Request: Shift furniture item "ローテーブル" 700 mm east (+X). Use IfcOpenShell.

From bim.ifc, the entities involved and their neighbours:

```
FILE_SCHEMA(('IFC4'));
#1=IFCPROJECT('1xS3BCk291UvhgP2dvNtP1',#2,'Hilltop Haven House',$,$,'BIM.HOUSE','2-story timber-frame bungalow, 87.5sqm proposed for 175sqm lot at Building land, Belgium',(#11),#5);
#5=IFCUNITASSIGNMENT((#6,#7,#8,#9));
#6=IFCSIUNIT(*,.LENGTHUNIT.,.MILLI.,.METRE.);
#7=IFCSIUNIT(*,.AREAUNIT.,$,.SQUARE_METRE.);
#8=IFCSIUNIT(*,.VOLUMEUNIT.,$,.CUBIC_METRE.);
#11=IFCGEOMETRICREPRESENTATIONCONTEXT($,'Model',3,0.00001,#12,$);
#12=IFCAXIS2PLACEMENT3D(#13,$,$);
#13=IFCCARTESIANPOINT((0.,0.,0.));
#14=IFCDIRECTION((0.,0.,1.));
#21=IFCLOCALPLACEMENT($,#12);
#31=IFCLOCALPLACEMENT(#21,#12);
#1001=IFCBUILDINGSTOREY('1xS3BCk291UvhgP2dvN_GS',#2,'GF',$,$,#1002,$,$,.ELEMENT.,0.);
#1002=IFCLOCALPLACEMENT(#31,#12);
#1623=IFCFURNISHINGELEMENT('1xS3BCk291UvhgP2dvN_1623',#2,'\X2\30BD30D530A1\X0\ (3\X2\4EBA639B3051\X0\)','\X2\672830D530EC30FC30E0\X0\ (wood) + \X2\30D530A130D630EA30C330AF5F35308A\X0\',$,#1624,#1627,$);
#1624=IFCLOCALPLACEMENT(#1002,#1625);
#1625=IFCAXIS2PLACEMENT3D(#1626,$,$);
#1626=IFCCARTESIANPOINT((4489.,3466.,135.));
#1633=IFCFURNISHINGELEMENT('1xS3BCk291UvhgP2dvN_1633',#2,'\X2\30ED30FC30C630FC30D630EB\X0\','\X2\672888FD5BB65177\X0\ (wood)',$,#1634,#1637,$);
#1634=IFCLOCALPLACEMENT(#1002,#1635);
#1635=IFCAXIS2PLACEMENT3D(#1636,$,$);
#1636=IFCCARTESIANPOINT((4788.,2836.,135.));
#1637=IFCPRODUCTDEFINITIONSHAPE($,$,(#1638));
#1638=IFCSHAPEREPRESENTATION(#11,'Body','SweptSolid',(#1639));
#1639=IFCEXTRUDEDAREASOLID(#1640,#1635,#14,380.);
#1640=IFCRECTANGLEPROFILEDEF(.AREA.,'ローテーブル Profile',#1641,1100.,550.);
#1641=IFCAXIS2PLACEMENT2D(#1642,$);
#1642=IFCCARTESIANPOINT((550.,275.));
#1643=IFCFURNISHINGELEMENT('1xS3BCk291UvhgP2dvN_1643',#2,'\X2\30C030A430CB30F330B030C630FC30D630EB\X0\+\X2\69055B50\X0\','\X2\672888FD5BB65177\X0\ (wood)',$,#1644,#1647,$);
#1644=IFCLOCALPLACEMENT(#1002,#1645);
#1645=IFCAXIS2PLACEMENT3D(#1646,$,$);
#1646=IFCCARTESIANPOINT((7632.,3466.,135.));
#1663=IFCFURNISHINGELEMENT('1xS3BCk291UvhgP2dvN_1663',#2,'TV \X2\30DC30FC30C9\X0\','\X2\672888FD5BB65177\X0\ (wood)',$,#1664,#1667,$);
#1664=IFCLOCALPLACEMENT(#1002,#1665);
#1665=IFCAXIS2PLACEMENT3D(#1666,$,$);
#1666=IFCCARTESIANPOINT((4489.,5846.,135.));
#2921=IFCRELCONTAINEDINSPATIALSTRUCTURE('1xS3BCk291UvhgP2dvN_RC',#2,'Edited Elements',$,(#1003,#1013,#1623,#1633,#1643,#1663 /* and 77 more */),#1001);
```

```python
import ifcopenshell
import ifcopenshell.api.geometry
import ifcopenshell.util.placement
import ifcopenshell.util.unit

model = ifcopenshell.open("bim.ifc")
unit_scale = ifcopenshell.util.unit.calculate_unit_scale(model)

item = model.by_guid("1xS3BCk291UvhgP2dvN_1633")
matrix = ifcopenshell.util.placement.get_local_placement(item.ObjectPlacement)
matrix[0, 3] += 0.7 / unit_scale
ifcopenshell.api.geometry.edit_object_placement(model, product=item, matrix=matrix, is_si=False)

print(ifcopenshell.util.placement.get_local_placement(item.ObjectPlacement).round(3) + 0.0)

model.write("bim_edited.ifc")
```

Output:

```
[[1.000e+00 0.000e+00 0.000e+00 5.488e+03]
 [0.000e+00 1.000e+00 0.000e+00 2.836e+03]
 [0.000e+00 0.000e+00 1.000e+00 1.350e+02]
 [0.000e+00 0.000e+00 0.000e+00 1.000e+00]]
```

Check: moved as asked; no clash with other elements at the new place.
